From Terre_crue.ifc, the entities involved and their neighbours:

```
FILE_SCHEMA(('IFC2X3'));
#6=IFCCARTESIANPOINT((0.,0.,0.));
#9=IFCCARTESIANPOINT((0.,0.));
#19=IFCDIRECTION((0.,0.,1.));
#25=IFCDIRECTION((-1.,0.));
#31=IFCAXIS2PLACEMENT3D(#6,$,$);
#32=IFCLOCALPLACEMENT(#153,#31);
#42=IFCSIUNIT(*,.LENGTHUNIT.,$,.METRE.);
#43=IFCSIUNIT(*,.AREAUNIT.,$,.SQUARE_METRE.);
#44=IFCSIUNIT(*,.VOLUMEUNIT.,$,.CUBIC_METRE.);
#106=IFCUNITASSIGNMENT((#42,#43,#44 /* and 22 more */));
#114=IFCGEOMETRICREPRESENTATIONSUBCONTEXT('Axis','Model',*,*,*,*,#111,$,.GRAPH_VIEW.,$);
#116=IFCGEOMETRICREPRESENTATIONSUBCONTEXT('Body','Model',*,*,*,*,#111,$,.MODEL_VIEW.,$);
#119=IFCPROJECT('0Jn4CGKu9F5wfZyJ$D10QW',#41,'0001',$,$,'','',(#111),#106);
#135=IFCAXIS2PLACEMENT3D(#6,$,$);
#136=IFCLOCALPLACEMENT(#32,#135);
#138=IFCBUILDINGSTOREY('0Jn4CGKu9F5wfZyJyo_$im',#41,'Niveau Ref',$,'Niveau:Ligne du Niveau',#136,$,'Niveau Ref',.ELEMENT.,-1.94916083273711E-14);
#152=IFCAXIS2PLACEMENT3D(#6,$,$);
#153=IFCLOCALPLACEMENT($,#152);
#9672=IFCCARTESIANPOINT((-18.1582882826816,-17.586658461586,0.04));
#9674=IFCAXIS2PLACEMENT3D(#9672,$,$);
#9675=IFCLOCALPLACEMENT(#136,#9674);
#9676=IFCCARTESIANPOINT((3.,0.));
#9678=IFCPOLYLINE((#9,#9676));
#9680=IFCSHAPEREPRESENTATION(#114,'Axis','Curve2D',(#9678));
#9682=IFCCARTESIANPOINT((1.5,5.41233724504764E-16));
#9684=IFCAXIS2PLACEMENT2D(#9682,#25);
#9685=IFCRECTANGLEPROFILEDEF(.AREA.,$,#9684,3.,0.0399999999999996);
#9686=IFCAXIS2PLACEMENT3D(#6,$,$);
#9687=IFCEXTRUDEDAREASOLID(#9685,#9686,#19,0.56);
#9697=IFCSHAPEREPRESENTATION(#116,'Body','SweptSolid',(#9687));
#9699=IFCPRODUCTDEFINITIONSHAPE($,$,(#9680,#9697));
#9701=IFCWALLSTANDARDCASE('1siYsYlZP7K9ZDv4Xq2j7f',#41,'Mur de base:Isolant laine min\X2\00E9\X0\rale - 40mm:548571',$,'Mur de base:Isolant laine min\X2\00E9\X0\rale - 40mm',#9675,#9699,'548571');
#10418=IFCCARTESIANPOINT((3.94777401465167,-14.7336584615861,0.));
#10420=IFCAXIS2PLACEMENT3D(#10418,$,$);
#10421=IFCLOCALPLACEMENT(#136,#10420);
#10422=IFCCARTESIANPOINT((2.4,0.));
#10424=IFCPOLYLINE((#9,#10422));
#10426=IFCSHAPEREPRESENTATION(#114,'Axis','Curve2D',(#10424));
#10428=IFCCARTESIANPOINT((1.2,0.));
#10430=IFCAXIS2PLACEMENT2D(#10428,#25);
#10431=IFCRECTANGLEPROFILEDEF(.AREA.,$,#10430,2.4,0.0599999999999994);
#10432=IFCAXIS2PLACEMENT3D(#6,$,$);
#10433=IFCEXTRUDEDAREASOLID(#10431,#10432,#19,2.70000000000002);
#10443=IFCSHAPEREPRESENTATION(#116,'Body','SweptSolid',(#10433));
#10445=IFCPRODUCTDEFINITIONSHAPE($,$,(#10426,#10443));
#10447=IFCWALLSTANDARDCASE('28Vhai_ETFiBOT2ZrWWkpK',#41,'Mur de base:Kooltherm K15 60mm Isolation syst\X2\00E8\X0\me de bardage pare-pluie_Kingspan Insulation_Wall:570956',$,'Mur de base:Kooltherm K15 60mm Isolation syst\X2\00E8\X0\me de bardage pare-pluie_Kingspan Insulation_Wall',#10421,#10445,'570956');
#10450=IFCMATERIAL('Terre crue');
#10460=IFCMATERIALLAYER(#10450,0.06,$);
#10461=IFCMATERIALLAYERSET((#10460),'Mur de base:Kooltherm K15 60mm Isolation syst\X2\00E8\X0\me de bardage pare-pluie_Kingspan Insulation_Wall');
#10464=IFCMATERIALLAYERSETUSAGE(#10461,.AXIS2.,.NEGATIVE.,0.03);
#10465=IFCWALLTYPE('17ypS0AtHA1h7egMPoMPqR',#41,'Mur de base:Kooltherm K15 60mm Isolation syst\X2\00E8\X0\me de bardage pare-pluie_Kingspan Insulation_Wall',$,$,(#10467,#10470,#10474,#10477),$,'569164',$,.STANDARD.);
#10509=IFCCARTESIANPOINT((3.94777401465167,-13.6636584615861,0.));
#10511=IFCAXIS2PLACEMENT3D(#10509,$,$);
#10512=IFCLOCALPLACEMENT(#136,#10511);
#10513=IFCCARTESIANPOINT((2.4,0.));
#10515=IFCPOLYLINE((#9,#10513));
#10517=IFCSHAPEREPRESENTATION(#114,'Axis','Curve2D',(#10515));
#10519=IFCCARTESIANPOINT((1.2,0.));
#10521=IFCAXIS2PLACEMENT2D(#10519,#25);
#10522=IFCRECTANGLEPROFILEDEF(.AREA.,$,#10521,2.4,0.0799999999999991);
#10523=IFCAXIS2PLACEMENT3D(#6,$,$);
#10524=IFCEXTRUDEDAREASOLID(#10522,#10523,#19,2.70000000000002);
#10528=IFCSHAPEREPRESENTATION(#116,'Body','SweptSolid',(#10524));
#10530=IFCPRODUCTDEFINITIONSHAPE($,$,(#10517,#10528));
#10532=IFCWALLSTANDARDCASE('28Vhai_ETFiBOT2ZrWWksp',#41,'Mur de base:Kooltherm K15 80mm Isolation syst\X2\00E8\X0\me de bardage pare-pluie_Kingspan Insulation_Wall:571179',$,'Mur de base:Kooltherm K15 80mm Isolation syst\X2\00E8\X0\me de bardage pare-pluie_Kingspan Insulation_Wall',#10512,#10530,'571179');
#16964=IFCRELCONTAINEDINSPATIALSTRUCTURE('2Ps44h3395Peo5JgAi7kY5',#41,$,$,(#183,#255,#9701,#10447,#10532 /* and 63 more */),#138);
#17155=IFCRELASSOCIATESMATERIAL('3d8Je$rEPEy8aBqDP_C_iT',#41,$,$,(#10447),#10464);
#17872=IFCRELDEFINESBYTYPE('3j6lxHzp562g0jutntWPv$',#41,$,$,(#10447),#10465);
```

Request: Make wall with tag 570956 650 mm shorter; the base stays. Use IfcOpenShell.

```python
import ifcopenshell
import ifcopenshell.geom
import ifcopenshell.util.representation
import ifcopenshell.util.shape

model = ifcopenshell.open("Terre_crue.ifc")
settings = ifcopenshell.geom.settings()


def volume(element):
    """Net volume in cubic metres, openings subtracted."""
    shape = ifcopenshell.geom.create_shape(settings, element)
    return ifcopenshell.util.shape.get_volume(shape.geometry)


wall = model.by_guid("28Vhai_ETFiBOT2ZrWWkpK")
before = volume(wall)

body = ifcopenshell.util.representation.get_representation(wall, "Model", "Body")
solid = body.Items[0]
old_height = solid.Depth
solid.Depth -= 0.65
after = volume(wall)

print(f"height {old_height:g} -> {solid.Depth:g}, volume {before:.3f} -> {after:.3f} m3")

model.write("Terre_crue_updated.ifc")
```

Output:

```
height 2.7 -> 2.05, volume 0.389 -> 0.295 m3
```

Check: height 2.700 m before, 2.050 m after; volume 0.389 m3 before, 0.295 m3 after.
